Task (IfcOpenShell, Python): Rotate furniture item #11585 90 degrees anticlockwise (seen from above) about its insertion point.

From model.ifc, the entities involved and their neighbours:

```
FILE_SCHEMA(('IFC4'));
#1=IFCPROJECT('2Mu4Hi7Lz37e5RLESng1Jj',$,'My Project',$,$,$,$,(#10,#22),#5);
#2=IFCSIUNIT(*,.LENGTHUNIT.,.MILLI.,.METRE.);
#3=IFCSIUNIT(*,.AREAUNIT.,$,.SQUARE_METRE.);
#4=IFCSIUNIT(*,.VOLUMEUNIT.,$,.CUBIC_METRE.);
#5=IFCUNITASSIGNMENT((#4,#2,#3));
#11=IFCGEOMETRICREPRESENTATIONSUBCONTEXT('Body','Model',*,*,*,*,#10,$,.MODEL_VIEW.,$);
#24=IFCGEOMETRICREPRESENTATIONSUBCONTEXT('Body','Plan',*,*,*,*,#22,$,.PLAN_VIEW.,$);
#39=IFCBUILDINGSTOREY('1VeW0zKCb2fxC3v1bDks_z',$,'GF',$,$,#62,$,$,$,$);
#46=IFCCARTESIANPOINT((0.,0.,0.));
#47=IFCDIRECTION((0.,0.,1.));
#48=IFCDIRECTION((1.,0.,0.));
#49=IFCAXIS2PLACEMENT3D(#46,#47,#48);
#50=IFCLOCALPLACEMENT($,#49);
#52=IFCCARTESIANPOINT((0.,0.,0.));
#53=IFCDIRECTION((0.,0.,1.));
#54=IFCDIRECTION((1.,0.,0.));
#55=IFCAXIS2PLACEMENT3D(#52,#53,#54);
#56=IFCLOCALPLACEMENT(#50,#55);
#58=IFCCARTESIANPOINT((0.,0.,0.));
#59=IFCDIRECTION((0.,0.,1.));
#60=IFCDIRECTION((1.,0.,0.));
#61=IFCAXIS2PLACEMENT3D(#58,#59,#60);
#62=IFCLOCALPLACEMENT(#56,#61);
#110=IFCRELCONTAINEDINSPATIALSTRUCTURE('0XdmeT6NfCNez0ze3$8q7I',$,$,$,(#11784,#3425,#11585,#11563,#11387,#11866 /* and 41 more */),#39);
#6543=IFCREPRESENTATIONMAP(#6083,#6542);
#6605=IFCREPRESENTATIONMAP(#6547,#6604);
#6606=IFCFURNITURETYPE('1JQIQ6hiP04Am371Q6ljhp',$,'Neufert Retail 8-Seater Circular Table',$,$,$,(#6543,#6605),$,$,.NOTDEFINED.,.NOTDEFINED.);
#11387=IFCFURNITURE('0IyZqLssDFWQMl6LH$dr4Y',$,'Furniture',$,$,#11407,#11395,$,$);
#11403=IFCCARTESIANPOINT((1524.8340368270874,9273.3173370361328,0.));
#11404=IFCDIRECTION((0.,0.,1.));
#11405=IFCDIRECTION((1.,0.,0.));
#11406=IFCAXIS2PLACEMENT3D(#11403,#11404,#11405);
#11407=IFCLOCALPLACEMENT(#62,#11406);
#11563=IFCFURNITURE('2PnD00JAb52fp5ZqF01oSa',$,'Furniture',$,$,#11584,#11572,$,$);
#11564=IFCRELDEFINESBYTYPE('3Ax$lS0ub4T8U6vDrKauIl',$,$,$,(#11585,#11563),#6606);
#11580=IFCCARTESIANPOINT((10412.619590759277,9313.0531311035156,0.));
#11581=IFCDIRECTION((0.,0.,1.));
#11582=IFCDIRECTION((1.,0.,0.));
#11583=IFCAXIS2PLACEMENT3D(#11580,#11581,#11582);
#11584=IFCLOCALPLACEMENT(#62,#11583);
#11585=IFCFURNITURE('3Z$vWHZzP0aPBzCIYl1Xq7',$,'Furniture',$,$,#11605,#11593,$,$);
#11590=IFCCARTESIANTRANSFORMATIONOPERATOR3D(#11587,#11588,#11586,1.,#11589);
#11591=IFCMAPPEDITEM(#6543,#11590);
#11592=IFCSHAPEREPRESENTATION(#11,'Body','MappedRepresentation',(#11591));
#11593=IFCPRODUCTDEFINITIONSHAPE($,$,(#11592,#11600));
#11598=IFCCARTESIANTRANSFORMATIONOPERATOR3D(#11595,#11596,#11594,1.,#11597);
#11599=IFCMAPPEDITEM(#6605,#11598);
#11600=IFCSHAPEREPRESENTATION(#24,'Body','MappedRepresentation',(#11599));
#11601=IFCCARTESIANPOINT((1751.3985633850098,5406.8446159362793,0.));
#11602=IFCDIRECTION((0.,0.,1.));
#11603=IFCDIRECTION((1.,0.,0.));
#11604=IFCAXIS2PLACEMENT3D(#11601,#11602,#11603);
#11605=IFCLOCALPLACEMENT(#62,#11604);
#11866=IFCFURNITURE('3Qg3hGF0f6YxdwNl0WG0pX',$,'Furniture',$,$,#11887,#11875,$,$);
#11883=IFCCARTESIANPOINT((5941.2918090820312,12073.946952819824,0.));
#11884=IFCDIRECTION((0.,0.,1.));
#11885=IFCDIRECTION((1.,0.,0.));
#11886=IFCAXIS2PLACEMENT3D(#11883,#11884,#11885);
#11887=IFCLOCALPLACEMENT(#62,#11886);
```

```python
import ifcopenshell
import ifcopenshell.api.geometry
import ifcopenshell.util.placement

model = ifcopenshell.open("model.ifc")

item = model.by_guid("3Z$vWHZzP0aPBzCIYl1Xq7")
matrix = ifcopenshell.util.placement.get_local_placement(item.ObjectPlacement)
matrix = matrix @ ifcopenshell.util.placement.rotation(90, "Z")
ifcopenshell.api.geometry.edit_object_placement(model, product=item, matrix=matrix, is_si=False)

print(ifcopenshell.util.placement.get_local_placement(item.ObjectPlacement).round(3) + 0.0)

model.write("model_v2.ifc")
```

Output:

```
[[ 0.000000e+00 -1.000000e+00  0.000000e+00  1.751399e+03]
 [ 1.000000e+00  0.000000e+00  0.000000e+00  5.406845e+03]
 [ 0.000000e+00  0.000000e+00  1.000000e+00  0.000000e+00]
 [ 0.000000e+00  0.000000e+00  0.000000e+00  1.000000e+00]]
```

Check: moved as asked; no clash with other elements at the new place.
